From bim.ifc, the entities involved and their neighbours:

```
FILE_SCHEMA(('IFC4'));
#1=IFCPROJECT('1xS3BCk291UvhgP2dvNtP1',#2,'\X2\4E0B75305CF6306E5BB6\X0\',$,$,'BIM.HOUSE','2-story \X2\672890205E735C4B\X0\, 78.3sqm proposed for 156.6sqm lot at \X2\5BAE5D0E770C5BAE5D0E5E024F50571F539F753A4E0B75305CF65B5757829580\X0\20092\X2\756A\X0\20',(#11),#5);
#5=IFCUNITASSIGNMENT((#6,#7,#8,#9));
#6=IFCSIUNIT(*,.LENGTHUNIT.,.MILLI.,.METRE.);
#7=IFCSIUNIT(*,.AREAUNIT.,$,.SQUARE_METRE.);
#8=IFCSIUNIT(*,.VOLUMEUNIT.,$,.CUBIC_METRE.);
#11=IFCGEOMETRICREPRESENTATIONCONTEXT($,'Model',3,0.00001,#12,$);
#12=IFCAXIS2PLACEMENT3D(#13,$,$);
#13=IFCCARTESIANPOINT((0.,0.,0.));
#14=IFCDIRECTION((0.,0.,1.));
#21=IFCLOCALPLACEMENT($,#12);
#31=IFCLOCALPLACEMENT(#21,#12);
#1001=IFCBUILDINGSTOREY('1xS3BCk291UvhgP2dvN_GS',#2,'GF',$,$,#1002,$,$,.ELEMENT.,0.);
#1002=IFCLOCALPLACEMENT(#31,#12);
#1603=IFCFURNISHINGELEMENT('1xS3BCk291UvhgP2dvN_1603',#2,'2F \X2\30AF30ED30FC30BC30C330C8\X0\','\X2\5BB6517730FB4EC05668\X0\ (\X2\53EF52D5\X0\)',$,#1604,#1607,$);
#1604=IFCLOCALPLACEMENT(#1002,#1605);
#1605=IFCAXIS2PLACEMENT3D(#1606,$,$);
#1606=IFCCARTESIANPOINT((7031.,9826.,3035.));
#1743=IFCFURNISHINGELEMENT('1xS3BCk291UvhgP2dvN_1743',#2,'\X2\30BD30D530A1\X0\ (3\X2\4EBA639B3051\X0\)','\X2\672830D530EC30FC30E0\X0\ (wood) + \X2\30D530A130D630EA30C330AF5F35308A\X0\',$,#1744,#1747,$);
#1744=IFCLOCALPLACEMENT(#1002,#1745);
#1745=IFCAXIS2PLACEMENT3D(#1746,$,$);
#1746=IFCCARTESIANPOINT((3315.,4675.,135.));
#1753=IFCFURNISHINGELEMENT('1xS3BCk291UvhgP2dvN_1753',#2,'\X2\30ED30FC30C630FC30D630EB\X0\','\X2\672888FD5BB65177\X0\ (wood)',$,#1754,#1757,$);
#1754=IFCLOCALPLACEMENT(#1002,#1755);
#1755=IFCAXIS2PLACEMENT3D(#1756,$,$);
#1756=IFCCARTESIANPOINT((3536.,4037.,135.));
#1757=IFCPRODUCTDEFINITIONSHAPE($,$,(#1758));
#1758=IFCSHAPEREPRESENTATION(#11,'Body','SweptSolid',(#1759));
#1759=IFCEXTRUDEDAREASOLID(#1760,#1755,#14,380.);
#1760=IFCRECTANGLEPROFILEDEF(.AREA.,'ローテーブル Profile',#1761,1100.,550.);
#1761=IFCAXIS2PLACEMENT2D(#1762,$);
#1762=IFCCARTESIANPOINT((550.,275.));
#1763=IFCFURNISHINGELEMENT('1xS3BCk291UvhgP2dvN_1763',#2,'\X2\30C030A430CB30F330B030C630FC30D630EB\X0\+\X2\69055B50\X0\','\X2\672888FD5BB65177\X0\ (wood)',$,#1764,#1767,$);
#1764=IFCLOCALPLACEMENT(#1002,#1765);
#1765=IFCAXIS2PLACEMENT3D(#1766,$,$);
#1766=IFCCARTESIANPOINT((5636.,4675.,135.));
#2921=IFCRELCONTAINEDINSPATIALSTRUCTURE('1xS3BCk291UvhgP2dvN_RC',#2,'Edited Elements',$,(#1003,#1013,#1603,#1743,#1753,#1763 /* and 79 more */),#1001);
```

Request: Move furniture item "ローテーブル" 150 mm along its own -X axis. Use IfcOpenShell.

```python
import ifcopenshell
import ifcopenshell.api.geometry
import ifcopenshell.util.placement

model = ifcopenshell.open("bim.ifc")

item = model.by_guid("1xS3BCk291UvhgP2dvN_1753")
matrix = ifcopenshell.util.placement.get_local_placement(item.ObjectPlacement)
matrix[:3, 3] -= matrix[:3, 0] * 150.0
ifcopenshell.api.geometry.edit_object_placement(model, product=item, matrix=matrix, is_si=False)

print(ifcopenshell.util.placement.get_local_placement(item.ObjectPlacement).round(3) + 0.0)

model.write("bim-out.ifc")
```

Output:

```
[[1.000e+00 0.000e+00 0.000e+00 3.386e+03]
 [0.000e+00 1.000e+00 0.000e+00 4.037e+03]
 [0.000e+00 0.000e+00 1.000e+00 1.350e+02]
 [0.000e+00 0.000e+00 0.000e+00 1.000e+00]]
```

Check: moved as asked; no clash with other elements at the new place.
